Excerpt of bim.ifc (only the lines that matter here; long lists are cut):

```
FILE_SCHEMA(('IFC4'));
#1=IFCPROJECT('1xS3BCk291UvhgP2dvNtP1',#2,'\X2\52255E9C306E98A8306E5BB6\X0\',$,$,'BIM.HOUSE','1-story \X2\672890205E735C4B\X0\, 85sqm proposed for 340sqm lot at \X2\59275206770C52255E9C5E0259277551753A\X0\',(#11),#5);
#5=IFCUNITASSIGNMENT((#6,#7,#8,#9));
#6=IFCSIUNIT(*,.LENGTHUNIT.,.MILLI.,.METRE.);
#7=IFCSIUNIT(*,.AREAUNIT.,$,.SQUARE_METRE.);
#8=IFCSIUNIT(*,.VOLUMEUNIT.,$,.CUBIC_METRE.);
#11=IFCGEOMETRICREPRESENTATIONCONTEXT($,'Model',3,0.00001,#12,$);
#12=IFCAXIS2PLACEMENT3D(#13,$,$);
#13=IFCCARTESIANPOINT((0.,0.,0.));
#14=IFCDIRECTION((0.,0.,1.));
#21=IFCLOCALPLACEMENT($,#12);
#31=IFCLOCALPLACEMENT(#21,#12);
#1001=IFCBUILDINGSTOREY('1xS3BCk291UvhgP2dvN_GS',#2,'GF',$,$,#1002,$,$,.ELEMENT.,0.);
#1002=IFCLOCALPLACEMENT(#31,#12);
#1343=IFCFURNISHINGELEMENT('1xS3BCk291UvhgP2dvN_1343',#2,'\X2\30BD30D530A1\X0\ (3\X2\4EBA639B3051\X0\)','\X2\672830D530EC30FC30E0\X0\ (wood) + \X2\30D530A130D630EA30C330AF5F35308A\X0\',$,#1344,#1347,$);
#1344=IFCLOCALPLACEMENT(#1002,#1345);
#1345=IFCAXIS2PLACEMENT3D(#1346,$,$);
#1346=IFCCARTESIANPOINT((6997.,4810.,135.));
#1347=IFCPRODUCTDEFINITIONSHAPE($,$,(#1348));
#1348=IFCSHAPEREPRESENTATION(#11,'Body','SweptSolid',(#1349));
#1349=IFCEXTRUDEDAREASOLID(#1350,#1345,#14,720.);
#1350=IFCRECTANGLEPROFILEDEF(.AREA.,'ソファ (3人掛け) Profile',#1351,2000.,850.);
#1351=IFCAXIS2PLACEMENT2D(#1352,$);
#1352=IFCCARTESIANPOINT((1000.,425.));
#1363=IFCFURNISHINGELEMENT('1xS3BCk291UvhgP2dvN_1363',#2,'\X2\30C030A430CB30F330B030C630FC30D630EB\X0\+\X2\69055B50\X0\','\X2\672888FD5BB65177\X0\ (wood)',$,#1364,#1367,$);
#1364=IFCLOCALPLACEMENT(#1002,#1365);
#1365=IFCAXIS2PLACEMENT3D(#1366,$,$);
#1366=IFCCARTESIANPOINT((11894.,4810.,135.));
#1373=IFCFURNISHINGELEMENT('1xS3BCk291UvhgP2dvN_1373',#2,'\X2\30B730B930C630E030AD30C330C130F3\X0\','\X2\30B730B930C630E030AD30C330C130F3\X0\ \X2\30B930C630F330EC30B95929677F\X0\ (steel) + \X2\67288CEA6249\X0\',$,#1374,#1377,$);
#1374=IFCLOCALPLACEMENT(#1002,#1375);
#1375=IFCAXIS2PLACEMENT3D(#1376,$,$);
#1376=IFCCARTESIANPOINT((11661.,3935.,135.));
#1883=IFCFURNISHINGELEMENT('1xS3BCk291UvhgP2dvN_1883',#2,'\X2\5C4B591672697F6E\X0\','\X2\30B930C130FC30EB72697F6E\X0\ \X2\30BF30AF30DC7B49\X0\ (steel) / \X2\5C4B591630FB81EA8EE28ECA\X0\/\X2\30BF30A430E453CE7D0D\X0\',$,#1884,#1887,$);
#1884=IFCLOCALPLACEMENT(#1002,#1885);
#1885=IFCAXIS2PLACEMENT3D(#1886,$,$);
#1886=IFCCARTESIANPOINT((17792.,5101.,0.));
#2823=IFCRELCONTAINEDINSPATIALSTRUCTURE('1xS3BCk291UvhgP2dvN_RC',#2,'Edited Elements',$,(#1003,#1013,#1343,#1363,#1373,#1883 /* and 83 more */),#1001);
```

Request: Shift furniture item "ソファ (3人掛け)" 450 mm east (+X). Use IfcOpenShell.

```python
import ifcopenshell
import ifcopenshell.api.geometry
import ifcopenshell.util.placement

model = ifcopenshell.open("bim.ifc")

item = model.by_id(1343)
matrix = ifcopenshell.util.placement.get_local_placement(item.ObjectPlacement)
matrix[0, 3] += 450.0
ifcopenshell.api.geometry.edit_object_placement(model, product=item, matrix=matrix, is_si=False)

print(ifcopenshell.util.placement.get_local_placement(item.ObjectPlacement).round(3) + 0.0)

model.write("bim_updated.ifc")
```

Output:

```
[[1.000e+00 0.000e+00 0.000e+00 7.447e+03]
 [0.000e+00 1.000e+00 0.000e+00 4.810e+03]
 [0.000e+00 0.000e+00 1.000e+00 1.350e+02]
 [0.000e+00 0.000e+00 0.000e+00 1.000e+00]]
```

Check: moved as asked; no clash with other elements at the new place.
